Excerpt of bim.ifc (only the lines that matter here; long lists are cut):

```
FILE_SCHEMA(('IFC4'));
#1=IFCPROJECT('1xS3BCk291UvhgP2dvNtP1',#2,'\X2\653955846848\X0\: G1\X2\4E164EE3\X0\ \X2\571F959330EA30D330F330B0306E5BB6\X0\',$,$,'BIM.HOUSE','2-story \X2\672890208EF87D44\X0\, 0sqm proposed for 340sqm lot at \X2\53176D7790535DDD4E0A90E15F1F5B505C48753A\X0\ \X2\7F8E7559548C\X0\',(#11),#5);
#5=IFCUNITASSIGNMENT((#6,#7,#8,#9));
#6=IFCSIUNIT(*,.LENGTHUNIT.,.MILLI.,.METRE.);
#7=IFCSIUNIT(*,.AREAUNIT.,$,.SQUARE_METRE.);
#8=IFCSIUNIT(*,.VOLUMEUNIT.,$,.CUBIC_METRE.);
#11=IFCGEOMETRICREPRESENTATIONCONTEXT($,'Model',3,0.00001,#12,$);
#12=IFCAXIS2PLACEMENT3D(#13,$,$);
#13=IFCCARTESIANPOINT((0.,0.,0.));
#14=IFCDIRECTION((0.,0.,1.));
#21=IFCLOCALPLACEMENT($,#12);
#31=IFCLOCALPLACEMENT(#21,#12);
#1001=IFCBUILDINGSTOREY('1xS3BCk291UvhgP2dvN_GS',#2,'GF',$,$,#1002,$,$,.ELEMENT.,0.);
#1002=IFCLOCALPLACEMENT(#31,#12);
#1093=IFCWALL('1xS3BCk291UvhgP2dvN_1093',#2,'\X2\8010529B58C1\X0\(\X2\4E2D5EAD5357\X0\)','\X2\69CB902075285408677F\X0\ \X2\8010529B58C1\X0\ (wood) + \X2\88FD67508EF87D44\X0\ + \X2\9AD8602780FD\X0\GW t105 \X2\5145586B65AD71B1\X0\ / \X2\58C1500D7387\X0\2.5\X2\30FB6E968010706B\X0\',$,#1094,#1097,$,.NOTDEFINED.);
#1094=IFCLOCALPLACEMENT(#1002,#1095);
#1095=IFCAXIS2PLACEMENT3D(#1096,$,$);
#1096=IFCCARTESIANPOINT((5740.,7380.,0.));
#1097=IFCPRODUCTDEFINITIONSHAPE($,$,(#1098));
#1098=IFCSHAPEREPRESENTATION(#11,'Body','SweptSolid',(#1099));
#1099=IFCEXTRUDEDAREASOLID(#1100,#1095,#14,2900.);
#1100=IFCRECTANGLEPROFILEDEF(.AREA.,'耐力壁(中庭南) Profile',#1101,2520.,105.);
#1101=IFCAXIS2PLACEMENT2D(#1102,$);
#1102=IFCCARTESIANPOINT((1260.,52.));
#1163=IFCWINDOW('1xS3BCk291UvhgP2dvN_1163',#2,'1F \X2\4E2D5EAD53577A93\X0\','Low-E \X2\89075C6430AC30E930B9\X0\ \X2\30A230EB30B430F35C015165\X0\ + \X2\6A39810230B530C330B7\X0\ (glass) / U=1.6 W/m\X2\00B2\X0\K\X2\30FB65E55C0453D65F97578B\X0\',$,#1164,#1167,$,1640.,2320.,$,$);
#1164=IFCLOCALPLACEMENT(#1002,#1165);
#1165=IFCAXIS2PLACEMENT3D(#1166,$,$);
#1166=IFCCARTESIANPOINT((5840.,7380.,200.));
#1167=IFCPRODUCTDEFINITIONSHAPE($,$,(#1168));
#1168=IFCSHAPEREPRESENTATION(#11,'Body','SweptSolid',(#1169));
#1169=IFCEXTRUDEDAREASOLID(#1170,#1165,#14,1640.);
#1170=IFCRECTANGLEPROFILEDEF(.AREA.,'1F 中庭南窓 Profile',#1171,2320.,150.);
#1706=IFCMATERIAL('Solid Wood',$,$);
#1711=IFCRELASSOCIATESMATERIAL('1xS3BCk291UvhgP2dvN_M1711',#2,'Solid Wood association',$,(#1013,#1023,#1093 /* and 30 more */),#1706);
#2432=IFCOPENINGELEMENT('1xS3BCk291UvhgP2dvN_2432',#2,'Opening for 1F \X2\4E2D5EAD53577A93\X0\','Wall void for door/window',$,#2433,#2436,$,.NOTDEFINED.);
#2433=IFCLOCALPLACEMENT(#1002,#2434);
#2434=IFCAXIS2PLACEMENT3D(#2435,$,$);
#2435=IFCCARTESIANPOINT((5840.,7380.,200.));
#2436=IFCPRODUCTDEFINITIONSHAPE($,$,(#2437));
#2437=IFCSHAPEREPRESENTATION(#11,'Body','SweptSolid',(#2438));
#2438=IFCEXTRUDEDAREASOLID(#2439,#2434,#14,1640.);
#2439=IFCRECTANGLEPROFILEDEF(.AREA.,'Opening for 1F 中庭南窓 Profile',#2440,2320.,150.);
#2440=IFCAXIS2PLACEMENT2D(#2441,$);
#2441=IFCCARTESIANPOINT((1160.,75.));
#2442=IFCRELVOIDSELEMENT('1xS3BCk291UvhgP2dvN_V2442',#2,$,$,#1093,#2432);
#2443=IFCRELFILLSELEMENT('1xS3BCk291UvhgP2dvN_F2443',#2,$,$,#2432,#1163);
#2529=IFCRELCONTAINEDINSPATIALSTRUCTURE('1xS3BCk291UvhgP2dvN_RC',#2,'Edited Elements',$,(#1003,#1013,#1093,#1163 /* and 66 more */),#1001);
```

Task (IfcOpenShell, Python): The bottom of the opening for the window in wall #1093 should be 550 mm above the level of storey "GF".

```python
import numpy as np
import ifcopenshell
import ifcopenshell.api.geometry
import ifcopenshell.geom
import ifcopenshell.util.element
import ifcopenshell.util.placement
import ifcopenshell.util.shape
import ifcopenshell.util.unit

model = ifcopenshell.open("bim.ifc")
unit_scale = ifcopenshell.util.unit.calculate_unit_scale(model)

window = model.by_guid("1xS3BCk291UvhgP2dvN_1163")
opening = window.FillsVoids[0].RelatingOpeningElement
storey = ifcopenshell.util.element.get_container(window, ifc_class="IfcBuildingStorey")
level = ifcopenshell.util.placement.get_local_placement(storey.ObjectPlacement)[2, 3]

# The opening's origin need not be at the sill, so measure its lowest point.
shape = ifcopenshell.geom.create_shape(ifcopenshell.geom.settings(), opening)
bottom = ifcopenshell.util.shape.get_shape_bottom_elevation(shape, shape.geometry) / unit_scale
dz = level + 550.0 - bottom

shift = np.array([0.0, 0.0, dz])
# The window is not placed relative to its opening, so move both.
for product in (opening, window):
    matrix = ifcopenshell.util.placement.get_local_placement(product.ObjectPlacement)
    matrix[:3, 3] += shift
    ifcopenshell.api.geometry.edit_object_placement(model, product=product, matrix=matrix, is_si=False)

print(f"moved by {dz * unit_scale:+.3f} m")

model.write("bim_v2.ifc")
```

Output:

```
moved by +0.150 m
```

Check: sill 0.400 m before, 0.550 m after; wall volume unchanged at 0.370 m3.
